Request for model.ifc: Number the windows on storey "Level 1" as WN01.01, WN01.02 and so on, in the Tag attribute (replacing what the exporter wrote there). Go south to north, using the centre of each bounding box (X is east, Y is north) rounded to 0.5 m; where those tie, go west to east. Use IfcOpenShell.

First a look at what the model holds.

```python
import ifcopenshell
import ifcopenshell.util.element
import ifcopenshell.util.placement

model = ifcopenshell.open("model.ifc")
print(model.schema)
storey = next(s for s in model.by_type("IfcBuildingStorey") if s.Name == "Level 1")
windows = [e for e in ifcopenshell.util.element.get_decomposition(storey) if e.is_a("IfcWindow")]
for e in sorted(windows, key=lambda e: e.id()):
    origin = ifcopenshell.util.placement.get_local_placement(e.ObjectPlacement)[:3, 3]
    print(e.id(), e.Tag, e.Name, origin.round(2) + 0.0, sep=" | ")
```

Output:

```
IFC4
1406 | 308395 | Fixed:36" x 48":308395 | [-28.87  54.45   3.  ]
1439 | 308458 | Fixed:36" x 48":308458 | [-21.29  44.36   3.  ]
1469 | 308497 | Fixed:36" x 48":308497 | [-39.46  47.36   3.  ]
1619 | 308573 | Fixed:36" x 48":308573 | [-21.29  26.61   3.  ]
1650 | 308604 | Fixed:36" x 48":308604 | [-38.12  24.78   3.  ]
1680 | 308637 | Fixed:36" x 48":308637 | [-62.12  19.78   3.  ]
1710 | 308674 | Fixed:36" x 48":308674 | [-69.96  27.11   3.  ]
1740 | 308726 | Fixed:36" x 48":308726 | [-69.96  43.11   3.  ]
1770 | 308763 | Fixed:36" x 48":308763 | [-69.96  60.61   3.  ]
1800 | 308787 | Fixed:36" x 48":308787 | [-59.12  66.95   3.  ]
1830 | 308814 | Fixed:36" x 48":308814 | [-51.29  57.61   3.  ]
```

```python
import ifcopenshell
import ifcopenshell.geom
import ifcopenshell.util.element
import ifcopenshell.util.shape

model = ifcopenshell.open("model.ifc")
settings = ifcopenshell.geom.settings()
settings.set("use-world-coords", True)


def centre(element):
    shape = ifcopenshell.geom.create_shape(settings, element)
    return ifcopenshell.util.shape.get_bbox_centroid(shape.geometry)


storey = next(s for s in model.by_type("IfcBuildingStorey") if s.Name == "Level 1")
windows = [e for e in ifcopenshell.util.element.get_decomposition(storey) if e.is_a("IfcWindow")]

# Insertion points can sit at a corner or the storey origin, so sort by the geometry (in metres).
centres = {e: centre(e) for e in windows}
windows.sort(key=lambda e: (round(centres[e][1] / 0.5), centres[e][0]))

for i, e in enumerate(windows, start=1):
    number = f"WN01.{i:02d}"
    e.Tag = number
    print(e.id(), number)

model.write("model-out.ifc")
```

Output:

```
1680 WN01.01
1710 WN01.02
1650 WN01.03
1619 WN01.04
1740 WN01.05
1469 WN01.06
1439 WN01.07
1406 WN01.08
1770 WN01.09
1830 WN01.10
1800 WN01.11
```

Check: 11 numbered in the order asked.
